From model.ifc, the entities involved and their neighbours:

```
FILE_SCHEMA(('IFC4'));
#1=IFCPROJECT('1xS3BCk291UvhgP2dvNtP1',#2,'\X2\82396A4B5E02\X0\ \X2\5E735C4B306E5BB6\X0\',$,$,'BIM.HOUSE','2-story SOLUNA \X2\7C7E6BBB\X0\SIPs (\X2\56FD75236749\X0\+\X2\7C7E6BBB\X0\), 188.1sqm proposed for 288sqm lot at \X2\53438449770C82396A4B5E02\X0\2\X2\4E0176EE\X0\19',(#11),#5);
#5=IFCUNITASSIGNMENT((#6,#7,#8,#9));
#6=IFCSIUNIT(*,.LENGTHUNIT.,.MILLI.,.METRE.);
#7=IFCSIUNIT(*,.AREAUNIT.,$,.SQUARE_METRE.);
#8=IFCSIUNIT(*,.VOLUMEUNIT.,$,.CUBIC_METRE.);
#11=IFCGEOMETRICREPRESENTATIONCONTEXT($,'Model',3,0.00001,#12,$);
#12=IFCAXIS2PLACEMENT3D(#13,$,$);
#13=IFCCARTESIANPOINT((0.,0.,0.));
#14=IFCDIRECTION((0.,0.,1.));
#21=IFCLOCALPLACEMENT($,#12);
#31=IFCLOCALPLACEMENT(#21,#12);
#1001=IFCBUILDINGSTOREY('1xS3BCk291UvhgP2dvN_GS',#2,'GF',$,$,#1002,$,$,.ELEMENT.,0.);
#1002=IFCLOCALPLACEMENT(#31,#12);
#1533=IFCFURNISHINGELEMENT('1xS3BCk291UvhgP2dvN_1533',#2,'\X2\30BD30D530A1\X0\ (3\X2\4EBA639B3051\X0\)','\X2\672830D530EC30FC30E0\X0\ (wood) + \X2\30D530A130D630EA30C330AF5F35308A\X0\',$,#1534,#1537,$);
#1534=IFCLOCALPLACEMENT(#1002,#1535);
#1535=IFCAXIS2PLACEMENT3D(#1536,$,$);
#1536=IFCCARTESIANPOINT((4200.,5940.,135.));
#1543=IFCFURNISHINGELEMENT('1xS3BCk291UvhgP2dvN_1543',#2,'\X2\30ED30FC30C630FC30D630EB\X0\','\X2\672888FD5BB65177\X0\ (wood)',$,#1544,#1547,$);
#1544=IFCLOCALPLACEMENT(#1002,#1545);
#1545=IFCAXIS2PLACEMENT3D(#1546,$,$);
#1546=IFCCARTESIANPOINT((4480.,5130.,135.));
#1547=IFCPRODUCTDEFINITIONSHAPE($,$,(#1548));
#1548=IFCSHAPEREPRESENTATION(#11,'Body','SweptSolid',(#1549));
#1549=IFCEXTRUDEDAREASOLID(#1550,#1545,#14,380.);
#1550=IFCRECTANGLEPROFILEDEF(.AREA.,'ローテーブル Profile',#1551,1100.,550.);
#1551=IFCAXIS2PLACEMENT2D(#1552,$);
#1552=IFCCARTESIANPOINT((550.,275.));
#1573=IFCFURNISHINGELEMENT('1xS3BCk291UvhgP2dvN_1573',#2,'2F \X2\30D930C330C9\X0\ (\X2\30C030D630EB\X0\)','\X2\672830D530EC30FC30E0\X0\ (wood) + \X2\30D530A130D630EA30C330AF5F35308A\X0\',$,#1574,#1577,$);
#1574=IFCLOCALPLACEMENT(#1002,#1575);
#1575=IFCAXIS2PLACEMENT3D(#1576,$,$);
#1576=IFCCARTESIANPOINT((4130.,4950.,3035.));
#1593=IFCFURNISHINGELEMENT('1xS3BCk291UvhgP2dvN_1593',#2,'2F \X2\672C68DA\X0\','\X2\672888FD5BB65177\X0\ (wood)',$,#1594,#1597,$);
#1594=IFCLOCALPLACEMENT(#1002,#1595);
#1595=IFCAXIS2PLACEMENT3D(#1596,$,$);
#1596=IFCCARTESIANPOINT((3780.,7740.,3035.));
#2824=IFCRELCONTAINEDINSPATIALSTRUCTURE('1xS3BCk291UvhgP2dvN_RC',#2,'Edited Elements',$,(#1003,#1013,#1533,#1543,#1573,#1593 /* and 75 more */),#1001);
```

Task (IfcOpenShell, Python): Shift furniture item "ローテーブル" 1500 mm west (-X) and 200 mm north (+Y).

```python
import ifcopenshell
import ifcopenshell.api.geometry
import ifcopenshell.util.placement

model = ifcopenshell.open("model.ifc")

item = model.by_guid("1xS3BCk291UvhgP2dvN_1543")
matrix = ifcopenshell.util.placement.get_local_placement(item.ObjectPlacement)
matrix[0, 3] -= 1500.0
matrix[1, 3] += 200.0
ifcopenshell.api.geometry.edit_object_placement(model, product=item, matrix=matrix, is_si=False)

print(ifcopenshell.util.placement.get_local_placement(item.ObjectPlacement).round(3) + 0.0)

model.write("model_rev.ifc")
```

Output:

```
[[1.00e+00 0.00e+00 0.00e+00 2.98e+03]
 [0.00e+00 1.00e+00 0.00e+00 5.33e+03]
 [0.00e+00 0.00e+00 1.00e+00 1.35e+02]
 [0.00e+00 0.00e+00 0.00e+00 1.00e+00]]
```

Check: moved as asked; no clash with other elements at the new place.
